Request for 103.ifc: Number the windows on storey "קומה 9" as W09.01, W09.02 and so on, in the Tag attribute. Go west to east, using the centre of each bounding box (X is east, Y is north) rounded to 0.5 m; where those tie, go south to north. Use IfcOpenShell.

First a look at what the model holds.

```python
import ifcopenshell
import ifcopenshell.util.element
import ifcopenshell.util.placement

model = ifcopenshell.open("103.ifc")
print(model.schema)
storey = next(s for s in model.by_type("IfcBuildingStorey") if s.Name == "קומה 9")
windows = [e for e in ifcopenshell.util.element.get_decomposition(storey) if e.is_a("IfcWindow")]
for e in sorted(windows, key=lambda e: e.id()):
    origin = ifcopenshell.util.placement.get_local_placement(e.ObjectPlacement)[:3, 3]
    print(e.id(), e.Tag, e.Name, origin.round(2) + 0.0, sep=" | ")
```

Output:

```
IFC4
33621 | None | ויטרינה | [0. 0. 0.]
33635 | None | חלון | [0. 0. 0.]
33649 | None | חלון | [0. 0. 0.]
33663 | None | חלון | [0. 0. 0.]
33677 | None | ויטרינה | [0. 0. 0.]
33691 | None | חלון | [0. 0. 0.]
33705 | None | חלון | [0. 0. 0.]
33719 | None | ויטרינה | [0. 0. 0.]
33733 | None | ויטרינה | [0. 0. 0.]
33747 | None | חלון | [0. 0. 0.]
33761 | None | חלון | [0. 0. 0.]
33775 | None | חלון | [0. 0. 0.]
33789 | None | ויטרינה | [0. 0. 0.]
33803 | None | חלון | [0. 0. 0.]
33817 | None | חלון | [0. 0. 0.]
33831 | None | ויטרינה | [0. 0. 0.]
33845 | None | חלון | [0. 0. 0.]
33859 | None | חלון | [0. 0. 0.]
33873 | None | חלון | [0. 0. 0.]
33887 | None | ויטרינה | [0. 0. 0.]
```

```python
import ifcopenshell
import ifcopenshell.geom
import ifcopenshell.util.element
import ifcopenshell.util.shape

model = ifcopenshell.open("103.ifc")
settings = ifcopenshell.geom.settings()
settings.set("use-world-coords", True)


def centre(element):
    shape = ifcopenshell.geom.create_shape(settings, element)
    return ifcopenshell.util.shape.get_bbox_centroid(shape.geometry)


storey = next(s for s in model.by_type("IfcBuildingStorey") if s.Name == "קומה 9")
windows = [e for e in ifcopenshell.util.element.get_decomposition(storey) if e.is_a("IfcWindow")]

# Insertion points can sit at a corner or the storey origin, so sort by the geometry (in metres).
centres = {e: centre(e) for e in windows}
windows.sort(key=lambda e: (round(centres[e][0] / 0.5), centres[e][1]))

for i, e in enumerate(windows, start=1):
    number = f"W09.{i:02d}"
    e.Tag = number
    print(e.id(), number)

model.write("103_rev.ifc")
```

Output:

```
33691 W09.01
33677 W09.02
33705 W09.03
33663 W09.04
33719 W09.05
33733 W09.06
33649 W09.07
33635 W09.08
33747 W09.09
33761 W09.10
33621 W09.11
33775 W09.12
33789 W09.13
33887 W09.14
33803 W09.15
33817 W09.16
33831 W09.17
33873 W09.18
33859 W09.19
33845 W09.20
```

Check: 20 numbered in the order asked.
